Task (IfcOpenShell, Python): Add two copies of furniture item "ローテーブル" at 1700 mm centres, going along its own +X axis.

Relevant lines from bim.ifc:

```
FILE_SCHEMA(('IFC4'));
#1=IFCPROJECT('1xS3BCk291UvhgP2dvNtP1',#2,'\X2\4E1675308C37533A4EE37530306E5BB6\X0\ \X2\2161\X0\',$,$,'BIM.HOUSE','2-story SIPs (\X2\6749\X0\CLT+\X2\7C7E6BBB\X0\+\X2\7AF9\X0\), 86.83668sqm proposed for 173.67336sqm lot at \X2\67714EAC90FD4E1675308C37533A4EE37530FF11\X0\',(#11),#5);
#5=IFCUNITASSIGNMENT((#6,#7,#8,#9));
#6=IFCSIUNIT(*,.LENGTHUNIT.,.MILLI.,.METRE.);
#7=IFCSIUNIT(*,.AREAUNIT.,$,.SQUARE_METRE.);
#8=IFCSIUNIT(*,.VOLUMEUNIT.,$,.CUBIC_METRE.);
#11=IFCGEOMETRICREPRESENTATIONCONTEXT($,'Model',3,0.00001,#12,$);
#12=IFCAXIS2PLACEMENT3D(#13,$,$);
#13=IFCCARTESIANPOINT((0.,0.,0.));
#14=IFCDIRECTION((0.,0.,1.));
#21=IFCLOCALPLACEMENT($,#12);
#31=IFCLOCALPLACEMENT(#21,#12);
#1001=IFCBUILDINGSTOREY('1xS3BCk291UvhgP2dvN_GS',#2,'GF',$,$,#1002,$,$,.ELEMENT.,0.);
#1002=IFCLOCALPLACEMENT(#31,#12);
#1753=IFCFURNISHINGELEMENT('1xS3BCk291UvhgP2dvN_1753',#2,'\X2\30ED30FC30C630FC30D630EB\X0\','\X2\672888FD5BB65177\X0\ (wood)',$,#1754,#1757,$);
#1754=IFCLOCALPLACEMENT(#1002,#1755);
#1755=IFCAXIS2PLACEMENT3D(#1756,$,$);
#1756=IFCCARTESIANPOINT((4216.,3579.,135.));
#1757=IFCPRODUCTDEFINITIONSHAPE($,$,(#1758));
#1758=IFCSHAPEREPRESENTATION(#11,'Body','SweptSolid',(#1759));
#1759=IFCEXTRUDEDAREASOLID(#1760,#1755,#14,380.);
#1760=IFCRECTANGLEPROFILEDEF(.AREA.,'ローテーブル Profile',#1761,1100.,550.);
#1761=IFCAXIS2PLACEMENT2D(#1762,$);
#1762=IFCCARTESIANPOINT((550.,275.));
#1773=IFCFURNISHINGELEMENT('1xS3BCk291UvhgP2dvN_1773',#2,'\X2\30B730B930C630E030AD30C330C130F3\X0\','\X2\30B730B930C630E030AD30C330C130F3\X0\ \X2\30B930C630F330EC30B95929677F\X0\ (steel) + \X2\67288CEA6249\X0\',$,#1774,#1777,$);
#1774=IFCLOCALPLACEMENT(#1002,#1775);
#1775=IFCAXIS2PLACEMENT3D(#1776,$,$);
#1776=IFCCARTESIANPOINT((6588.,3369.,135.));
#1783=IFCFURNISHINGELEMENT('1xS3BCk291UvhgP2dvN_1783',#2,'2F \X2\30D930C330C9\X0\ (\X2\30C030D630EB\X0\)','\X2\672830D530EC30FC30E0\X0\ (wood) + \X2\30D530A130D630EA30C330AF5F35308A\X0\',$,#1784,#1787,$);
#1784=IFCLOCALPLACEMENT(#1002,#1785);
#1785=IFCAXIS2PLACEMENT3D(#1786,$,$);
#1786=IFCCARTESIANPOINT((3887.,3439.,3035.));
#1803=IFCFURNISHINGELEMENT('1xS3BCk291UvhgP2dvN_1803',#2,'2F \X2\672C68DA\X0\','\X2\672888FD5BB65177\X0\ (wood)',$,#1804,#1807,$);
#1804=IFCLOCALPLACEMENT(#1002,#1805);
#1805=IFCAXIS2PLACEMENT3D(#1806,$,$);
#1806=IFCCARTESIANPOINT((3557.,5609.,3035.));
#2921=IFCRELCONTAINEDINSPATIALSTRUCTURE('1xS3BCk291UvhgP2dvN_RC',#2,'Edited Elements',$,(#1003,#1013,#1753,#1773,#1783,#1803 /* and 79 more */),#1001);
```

```python
import ifcopenshell
import ifcopenshell.api.geometry
import ifcopenshell.api.root
import ifcopenshell.util.element
import ifcopenshell.util.placement
import ifcopenshell.util.unit

model = ifcopenshell.open("bim.ifc")
unit_scale = ifcopenshell.util.unit.calculate_unit_scale(model)


def reuse_history(source, copy):
    """copy_class also copies each property set's owner history, people and application; keep the originals."""
    for rel in copy.IsDefinedBy:
        if rel.is_a("IfcRelDefinesByProperties") and (history := rel.RelatingPropertyDefinition.OwnerHistory):
            rel.RelatingPropertyDefinition.OwnerHistory = source.OwnerHistory
            ifcopenshell.util.element.remove_deep2(model, history)


source = model.by_guid("1xS3BCk291UvhgP2dvN_1753")
base = ifcopenshell.util.placement.get_local_placement(source.ObjectPlacement)
step = base[:3, 0] * 1.7 / unit_scale

for i in range(1, 3):
    copy = ifcopenshell.api.root.copy_class(model, product=source)
    copy.Representation = ifcopenshell.util.element.copy_deep(
        model, source.Representation, exclude=["IfcGeometricRepresentationContext", "IfcRepresentationMap"]
    )
    reuse_history(source, copy)
    matrix = base.copy()
    matrix[:3, 3] += i * step
    print("added at", matrix[:3, 3].round(3) + 0.0)
    ifcopenshell.api.geometry.edit_object_placement(model, product=copy, matrix=matrix, is_si=False)

model.write("bim_rev.ifc")
```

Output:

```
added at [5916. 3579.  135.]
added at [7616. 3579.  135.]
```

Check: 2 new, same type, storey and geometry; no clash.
